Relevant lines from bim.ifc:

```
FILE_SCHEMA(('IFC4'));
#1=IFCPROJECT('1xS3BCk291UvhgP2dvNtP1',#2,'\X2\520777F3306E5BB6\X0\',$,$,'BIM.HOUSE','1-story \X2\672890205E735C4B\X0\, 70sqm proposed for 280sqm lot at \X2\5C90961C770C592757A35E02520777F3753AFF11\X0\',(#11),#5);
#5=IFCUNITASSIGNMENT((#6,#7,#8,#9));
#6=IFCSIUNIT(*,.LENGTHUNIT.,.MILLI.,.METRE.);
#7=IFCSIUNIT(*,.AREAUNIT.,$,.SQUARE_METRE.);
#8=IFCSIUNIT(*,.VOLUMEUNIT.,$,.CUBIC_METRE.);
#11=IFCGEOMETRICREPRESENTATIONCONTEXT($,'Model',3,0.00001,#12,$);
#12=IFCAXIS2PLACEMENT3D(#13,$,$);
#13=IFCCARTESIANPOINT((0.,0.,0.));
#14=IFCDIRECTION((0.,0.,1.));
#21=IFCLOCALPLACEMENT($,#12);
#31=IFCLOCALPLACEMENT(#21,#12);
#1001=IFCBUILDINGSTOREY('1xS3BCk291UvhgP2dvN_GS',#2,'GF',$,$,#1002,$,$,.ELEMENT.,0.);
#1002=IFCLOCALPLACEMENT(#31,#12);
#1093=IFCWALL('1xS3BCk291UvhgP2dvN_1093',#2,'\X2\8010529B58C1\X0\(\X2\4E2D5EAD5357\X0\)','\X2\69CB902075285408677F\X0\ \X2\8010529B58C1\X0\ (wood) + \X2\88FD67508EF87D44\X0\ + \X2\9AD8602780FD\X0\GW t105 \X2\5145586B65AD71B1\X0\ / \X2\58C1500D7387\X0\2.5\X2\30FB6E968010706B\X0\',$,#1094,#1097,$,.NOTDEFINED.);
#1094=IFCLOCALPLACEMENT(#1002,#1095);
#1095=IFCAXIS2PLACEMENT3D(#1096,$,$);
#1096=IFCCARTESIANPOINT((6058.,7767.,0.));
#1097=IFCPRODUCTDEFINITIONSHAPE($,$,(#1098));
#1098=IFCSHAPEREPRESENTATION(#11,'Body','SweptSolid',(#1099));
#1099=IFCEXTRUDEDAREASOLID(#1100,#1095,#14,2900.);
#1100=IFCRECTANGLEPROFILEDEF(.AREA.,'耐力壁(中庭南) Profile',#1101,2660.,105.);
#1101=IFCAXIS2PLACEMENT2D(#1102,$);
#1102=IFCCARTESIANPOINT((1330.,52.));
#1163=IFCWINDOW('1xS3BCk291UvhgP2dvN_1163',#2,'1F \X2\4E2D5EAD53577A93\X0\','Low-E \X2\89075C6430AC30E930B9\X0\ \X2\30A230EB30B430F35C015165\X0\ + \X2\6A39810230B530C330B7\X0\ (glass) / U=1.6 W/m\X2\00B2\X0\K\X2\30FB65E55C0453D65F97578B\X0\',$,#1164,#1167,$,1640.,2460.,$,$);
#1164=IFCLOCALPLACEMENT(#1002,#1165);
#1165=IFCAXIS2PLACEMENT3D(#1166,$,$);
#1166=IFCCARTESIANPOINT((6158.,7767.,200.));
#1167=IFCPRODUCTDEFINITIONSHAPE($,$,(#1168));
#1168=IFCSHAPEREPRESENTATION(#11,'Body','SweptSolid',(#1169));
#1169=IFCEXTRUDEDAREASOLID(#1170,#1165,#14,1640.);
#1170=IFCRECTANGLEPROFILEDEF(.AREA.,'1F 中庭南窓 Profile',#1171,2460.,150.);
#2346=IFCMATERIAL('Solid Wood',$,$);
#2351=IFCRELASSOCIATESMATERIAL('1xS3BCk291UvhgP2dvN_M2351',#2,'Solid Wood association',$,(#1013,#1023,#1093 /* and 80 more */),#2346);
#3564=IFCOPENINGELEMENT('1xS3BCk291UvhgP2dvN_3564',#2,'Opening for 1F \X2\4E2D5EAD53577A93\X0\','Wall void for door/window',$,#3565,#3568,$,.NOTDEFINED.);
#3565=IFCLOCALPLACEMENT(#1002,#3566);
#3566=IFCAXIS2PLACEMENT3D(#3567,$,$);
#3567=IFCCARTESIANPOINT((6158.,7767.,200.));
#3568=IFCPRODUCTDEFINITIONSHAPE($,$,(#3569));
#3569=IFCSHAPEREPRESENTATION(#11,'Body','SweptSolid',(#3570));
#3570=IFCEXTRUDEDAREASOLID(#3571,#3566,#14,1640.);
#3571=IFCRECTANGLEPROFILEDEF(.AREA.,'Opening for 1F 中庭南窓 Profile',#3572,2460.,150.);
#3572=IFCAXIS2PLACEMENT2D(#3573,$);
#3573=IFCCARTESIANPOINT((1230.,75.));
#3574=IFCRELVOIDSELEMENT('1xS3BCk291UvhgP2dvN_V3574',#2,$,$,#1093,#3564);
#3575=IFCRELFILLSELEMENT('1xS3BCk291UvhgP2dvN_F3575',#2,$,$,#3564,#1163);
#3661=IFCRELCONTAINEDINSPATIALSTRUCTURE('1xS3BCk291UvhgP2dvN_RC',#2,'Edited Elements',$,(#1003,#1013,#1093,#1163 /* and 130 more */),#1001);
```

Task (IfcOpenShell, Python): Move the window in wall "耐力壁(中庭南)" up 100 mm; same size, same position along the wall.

```python
import numpy as np
import ifcopenshell
import ifcopenshell.api.geometry
import ifcopenshell.util.placement
import ifcopenshell.util.unit

model = ifcopenshell.open("bim.ifc")
unit_scale = ifcopenshell.util.unit.calculate_unit_scale(model)

window = model.by_id(1163)
opening = window.FillsVoids[0].RelatingOpeningElement
dz = 0.1 / unit_scale

shift = np.array([0.0, 0.0, dz])
# The window is not placed relative to its opening, so move both.
for product in (opening, window):
    matrix = ifcopenshell.util.placement.get_local_placement(product.ObjectPlacement)
    matrix[:3, 3] += shift
    ifcopenshell.api.geometry.edit_object_placement(model, product=product, matrix=matrix, is_si=False)

print(f"moved by {dz * unit_scale:+.3f} m")

model.write("bim-out.ifc")
```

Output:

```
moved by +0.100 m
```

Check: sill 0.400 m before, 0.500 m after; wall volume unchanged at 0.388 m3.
